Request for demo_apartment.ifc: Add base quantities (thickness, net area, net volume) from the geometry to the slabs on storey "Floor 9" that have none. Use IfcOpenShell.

First a look at what the model holds.

```python
import ifcopenshell
import ifcopenshell.util.element
import ifcopenshell.util.unit

model = ifcopenshell.open("demo_apartment.ifc")
print(model.schema)
for unit_type in ("LENGTHUNIT", "AREAUNIT", "VOLUMEUNIT"):
    print(unit_type, ifcopenshell.util.unit.calculate_unit_scale(model, unit_type))
storey = next(s for s in model.by_type("IfcBuildingStorey") if s.Name == "Floor 9")
slabs = [e for e in ifcopenshell.util.element.get_decomposition(storey) if e.is_a("IfcSlab")]
for e in sorted(slabs, key=lambda e: e.id()):
    print(e.id(), e.is_a(), e.Name, list(ifcopenshell.util.element.get_psets(e, qtos_only=True)), sep=" | ")
```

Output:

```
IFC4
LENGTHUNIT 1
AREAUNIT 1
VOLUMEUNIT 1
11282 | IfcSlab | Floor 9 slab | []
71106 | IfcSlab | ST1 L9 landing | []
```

```python
import ifcopenshell
import ifcopenshell.api.pset
import ifcopenshell.geom
import ifcopenshell.util.element
import ifcopenshell.util.shape
import ifcopenshell.util.unit

model = ifcopenshell.open("demo_apartment.ifc")
unit_scale = ifcopenshell.util.unit.calculate_unit_scale(model)
area_scale = ifcopenshell.util.unit.calculate_unit_scale(model, "AREAUNIT")
volume_scale = ifcopenshell.util.unit.calculate_unit_scale(model, "VOLUMEUNIT")
settings = ifcopenshell.geom.settings()

storey = next(s for s in model.by_type("IfcBuildingStorey") if s.Name == "Floor 9")
slabs = [e for e in ifcopenshell.util.element.get_decomposition(storey) if e.is_a("IfcSlab")]

for e in sorted(slabs, key=lambda e: e.id()):
    if ifcopenshell.util.element.get_psets(e, qtos_only=True, should_inherit=False):
        continue
    # Geometry comes back in metres, in the element's own axes.
    shape = ifcopenshell.geom.create_shape(settings, e)
    values = {
        "Width": ifcopenshell.util.shape.get_z(shape.geometry) / unit_scale,
        "NetArea": ifcopenshell.util.shape.get_footprint_area(shape.geometry) / area_scale,
        "NetVolume": ifcopenshell.util.shape.get_volume(shape.geometry) / volume_scale,
    }
    qto = ifcopenshell.api.pset.add_qto(model, product=e, name="Qto_SlabBaseQuantities")
    ifcopenshell.api.pset.edit_qto(model, qto=qto, properties=values)
    print(e.id(), {k: round(v, 3) for k, v in values.items()})

model.write("demo_apartment-out.ifc")
```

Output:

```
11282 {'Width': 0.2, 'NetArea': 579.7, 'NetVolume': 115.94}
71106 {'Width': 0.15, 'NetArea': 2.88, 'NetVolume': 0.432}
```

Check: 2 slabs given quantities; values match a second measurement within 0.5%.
